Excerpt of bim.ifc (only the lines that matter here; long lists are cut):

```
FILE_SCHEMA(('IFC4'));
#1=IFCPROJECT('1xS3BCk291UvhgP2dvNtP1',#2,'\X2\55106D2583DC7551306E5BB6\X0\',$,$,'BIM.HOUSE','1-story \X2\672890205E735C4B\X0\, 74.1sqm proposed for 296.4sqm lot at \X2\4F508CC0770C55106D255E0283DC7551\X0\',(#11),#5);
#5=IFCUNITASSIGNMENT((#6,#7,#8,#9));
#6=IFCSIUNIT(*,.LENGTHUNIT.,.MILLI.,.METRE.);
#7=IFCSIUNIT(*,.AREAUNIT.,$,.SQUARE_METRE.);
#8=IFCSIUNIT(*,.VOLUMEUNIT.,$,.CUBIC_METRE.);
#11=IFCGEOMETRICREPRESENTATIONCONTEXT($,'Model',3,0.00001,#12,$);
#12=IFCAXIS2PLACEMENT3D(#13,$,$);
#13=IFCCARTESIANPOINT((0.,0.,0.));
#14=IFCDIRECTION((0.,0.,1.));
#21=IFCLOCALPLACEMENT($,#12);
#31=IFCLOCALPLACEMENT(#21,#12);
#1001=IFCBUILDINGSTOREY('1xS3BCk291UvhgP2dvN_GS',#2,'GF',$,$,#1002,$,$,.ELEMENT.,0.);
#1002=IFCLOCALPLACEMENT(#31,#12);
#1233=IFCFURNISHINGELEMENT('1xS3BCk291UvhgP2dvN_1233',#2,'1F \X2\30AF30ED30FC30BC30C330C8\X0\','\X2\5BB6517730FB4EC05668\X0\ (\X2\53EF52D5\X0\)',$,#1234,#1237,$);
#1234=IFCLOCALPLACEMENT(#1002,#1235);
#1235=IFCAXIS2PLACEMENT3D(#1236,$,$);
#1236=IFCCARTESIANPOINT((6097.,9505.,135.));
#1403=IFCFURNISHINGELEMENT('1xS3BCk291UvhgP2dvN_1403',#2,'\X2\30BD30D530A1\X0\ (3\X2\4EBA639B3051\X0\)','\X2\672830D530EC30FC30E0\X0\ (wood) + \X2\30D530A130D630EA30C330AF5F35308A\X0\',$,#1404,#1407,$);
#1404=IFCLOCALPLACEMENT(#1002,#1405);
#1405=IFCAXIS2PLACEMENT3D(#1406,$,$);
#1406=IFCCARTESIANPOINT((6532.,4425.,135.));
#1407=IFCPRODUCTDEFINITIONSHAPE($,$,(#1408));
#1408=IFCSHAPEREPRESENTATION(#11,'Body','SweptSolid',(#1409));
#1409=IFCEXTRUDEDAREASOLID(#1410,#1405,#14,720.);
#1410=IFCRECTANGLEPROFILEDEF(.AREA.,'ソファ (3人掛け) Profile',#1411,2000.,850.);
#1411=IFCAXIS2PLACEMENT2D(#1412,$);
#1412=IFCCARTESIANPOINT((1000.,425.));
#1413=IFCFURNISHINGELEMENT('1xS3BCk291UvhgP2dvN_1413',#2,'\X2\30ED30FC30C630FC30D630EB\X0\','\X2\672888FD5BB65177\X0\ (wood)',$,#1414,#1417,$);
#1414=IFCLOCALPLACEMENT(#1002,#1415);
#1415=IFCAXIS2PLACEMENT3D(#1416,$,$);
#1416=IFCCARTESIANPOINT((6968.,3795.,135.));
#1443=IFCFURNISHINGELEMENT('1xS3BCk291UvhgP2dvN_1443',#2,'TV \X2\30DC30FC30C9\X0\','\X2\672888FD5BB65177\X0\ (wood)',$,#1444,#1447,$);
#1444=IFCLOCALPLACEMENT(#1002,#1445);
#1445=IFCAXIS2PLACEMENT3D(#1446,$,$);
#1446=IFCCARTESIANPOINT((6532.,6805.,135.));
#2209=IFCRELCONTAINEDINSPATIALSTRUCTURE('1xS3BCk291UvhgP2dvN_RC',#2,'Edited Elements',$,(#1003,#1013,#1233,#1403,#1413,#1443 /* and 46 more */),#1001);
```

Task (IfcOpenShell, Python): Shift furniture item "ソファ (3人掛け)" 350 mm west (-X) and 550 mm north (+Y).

```python
import ifcopenshell
import ifcopenshell.api.geometry
import ifcopenshell.util.placement
import ifcopenshell.util.unit

model = ifcopenshell.open("bim.ifc")
unit_scale = ifcopenshell.util.unit.calculate_unit_scale(model)

item = model.by_guid("1xS3BCk291UvhgP2dvN_1403")
matrix = ifcopenshell.util.placement.get_local_placement(item.ObjectPlacement)
matrix[0, 3] -= 0.35 / unit_scale
matrix[1, 3] += 0.55 / unit_scale
ifcopenshell.api.geometry.edit_object_placement(model, product=item, matrix=matrix, is_si=False)

print(ifcopenshell.util.placement.get_local_placement(item.ObjectPlacement).round(3) + 0.0)

model.write("bim_v2.ifc")
```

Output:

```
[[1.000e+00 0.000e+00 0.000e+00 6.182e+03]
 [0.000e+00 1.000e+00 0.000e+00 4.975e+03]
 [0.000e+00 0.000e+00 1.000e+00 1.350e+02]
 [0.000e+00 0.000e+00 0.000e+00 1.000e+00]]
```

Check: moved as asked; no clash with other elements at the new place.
